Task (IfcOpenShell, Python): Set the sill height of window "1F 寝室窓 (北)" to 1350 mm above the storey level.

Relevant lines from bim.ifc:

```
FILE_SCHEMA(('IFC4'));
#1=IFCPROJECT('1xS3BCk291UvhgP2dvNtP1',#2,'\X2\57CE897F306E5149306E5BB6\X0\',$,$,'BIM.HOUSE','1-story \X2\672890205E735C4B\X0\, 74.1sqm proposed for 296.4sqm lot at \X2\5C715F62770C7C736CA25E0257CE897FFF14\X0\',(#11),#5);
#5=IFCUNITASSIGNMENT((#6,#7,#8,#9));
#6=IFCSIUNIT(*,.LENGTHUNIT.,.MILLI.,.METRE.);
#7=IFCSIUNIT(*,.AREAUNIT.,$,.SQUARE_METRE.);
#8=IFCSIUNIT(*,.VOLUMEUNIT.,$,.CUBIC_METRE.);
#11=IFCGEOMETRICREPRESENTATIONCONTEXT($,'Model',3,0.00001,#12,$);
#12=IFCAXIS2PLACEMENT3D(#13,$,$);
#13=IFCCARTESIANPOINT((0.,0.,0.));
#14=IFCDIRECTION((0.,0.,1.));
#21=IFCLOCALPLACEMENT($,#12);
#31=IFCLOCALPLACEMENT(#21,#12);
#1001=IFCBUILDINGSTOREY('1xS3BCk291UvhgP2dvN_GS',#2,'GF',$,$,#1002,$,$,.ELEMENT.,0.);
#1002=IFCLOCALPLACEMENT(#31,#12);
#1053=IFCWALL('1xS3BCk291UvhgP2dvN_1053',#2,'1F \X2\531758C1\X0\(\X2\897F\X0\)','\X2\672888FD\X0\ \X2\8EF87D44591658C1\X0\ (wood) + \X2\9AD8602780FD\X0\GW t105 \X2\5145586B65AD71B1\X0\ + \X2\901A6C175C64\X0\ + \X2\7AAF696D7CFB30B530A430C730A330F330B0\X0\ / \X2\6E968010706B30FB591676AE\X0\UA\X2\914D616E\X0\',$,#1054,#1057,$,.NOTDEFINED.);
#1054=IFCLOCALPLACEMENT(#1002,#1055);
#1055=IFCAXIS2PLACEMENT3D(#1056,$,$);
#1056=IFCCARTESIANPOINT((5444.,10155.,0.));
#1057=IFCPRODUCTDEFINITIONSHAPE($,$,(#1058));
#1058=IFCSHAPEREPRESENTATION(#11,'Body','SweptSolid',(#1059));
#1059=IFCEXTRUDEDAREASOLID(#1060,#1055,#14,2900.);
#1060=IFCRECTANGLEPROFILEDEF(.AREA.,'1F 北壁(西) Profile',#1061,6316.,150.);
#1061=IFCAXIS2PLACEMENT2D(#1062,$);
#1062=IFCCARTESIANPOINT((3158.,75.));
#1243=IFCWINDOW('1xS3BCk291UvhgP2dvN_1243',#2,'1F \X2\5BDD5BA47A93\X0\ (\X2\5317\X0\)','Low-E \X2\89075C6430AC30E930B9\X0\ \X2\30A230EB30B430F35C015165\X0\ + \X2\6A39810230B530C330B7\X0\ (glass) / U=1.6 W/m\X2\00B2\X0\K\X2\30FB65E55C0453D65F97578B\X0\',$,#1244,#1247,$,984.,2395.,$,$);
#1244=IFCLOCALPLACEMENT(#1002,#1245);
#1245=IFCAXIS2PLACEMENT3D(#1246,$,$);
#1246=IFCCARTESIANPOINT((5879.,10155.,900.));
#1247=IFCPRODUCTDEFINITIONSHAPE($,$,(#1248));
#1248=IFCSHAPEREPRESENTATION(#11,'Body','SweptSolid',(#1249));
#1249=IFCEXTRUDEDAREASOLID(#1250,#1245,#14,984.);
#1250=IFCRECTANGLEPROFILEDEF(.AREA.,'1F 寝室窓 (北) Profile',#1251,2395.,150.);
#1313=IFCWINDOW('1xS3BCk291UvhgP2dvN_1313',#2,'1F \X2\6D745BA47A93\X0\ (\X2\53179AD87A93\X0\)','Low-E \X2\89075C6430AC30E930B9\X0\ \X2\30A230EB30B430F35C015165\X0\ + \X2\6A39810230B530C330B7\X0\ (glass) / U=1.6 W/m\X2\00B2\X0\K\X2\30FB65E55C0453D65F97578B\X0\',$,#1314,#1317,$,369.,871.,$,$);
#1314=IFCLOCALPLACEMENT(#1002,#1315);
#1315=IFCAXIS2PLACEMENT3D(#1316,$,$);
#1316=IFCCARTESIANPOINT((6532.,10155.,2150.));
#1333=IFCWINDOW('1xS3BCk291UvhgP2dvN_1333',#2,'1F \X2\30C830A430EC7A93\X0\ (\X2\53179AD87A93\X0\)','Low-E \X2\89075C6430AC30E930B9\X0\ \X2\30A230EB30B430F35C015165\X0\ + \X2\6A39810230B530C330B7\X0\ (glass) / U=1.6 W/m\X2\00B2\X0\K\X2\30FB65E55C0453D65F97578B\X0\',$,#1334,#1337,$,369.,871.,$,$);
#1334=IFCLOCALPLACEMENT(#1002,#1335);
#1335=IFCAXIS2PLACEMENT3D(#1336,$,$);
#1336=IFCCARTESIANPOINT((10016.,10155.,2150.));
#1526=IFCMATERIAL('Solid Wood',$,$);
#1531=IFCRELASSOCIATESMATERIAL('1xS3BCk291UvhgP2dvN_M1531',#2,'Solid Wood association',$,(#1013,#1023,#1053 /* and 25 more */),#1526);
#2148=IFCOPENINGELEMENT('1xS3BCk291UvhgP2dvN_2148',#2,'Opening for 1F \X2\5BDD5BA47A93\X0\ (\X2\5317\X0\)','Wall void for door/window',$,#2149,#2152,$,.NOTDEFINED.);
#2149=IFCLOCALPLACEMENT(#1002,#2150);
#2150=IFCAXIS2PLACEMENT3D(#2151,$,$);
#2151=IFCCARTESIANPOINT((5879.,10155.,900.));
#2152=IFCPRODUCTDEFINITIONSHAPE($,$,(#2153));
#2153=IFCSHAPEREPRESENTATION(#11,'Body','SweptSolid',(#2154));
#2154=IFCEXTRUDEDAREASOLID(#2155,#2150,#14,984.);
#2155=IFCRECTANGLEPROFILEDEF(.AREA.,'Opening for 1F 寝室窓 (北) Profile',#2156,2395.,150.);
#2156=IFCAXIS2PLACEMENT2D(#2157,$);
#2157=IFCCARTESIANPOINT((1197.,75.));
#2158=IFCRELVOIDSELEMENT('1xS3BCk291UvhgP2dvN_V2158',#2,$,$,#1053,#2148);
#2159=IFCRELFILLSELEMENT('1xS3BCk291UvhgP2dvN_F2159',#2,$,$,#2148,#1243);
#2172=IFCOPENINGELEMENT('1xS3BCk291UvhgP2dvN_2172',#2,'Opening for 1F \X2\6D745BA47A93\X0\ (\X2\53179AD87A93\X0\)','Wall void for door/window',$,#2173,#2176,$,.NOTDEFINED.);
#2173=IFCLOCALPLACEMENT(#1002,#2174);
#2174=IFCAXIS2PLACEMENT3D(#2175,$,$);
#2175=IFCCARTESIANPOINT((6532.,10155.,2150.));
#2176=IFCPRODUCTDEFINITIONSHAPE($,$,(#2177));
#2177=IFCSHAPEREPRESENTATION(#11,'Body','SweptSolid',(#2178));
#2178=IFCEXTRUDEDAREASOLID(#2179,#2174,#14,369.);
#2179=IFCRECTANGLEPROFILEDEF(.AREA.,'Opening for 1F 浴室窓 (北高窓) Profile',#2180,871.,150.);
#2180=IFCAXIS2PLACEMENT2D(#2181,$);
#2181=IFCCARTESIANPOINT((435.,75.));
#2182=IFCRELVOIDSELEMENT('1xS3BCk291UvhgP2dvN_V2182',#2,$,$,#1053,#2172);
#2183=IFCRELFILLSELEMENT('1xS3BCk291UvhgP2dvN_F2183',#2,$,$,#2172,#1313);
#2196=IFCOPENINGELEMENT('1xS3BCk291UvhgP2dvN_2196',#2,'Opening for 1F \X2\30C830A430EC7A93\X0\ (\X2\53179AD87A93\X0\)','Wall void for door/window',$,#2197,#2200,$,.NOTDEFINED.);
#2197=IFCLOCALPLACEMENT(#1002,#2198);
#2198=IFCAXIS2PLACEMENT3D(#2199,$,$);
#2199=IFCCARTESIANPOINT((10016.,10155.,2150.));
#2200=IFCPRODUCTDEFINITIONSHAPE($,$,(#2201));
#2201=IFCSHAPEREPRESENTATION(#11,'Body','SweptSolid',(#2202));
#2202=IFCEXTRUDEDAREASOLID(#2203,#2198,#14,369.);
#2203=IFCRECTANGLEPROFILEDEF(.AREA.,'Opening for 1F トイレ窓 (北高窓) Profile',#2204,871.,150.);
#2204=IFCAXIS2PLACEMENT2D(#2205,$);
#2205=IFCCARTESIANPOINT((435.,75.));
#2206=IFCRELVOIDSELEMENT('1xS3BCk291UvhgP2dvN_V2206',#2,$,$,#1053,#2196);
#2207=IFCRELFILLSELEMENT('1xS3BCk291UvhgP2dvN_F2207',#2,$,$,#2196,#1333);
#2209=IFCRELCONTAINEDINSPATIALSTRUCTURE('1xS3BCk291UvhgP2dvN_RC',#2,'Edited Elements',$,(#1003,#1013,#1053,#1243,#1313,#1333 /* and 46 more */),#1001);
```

```python
import numpy as np
import ifcopenshell
import ifcopenshell.api.geometry
import ifcopenshell.geom
import ifcopenshell.util.element
import ifcopenshell.util.placement
import ifcopenshell.util.shape
import ifcopenshell.util.unit

model = ifcopenshell.open("bim.ifc")
unit_scale = ifcopenshell.util.unit.calculate_unit_scale(model)

window = model.by_id(1243)
opening = window.FillsVoids[0].RelatingOpeningElement
storey = ifcopenshell.util.element.get_container(window, ifc_class="IfcBuildingStorey")
level = ifcopenshell.util.placement.get_local_placement(storey.ObjectPlacement)[2, 3]

# The opening's origin need not be at the sill, so measure its lowest point.
shape = ifcopenshell.geom.create_shape(ifcopenshell.geom.settings(), opening)
bottom = ifcopenshell.util.shape.get_shape_bottom_elevation(shape, shape.geometry) / unit_scale
dz = level + 1.35 / unit_scale - bottom

shift = np.array([0.0, 0.0, dz])
# The window is not placed relative to its opening, so move both.
for product in (opening, window):
    matrix = ifcopenshell.util.placement.get_local_placement(product.ObjectPlacement)
    matrix[:3, 3] += shift
    ifcopenshell.api.geometry.edit_object_placement(model, product=product, matrix=matrix, is_si=False)

print(f"moved by {dz * unit_scale:+.3f} m")

model.write("bim-out.ifc")
```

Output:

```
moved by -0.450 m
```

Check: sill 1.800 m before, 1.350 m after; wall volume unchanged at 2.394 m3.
